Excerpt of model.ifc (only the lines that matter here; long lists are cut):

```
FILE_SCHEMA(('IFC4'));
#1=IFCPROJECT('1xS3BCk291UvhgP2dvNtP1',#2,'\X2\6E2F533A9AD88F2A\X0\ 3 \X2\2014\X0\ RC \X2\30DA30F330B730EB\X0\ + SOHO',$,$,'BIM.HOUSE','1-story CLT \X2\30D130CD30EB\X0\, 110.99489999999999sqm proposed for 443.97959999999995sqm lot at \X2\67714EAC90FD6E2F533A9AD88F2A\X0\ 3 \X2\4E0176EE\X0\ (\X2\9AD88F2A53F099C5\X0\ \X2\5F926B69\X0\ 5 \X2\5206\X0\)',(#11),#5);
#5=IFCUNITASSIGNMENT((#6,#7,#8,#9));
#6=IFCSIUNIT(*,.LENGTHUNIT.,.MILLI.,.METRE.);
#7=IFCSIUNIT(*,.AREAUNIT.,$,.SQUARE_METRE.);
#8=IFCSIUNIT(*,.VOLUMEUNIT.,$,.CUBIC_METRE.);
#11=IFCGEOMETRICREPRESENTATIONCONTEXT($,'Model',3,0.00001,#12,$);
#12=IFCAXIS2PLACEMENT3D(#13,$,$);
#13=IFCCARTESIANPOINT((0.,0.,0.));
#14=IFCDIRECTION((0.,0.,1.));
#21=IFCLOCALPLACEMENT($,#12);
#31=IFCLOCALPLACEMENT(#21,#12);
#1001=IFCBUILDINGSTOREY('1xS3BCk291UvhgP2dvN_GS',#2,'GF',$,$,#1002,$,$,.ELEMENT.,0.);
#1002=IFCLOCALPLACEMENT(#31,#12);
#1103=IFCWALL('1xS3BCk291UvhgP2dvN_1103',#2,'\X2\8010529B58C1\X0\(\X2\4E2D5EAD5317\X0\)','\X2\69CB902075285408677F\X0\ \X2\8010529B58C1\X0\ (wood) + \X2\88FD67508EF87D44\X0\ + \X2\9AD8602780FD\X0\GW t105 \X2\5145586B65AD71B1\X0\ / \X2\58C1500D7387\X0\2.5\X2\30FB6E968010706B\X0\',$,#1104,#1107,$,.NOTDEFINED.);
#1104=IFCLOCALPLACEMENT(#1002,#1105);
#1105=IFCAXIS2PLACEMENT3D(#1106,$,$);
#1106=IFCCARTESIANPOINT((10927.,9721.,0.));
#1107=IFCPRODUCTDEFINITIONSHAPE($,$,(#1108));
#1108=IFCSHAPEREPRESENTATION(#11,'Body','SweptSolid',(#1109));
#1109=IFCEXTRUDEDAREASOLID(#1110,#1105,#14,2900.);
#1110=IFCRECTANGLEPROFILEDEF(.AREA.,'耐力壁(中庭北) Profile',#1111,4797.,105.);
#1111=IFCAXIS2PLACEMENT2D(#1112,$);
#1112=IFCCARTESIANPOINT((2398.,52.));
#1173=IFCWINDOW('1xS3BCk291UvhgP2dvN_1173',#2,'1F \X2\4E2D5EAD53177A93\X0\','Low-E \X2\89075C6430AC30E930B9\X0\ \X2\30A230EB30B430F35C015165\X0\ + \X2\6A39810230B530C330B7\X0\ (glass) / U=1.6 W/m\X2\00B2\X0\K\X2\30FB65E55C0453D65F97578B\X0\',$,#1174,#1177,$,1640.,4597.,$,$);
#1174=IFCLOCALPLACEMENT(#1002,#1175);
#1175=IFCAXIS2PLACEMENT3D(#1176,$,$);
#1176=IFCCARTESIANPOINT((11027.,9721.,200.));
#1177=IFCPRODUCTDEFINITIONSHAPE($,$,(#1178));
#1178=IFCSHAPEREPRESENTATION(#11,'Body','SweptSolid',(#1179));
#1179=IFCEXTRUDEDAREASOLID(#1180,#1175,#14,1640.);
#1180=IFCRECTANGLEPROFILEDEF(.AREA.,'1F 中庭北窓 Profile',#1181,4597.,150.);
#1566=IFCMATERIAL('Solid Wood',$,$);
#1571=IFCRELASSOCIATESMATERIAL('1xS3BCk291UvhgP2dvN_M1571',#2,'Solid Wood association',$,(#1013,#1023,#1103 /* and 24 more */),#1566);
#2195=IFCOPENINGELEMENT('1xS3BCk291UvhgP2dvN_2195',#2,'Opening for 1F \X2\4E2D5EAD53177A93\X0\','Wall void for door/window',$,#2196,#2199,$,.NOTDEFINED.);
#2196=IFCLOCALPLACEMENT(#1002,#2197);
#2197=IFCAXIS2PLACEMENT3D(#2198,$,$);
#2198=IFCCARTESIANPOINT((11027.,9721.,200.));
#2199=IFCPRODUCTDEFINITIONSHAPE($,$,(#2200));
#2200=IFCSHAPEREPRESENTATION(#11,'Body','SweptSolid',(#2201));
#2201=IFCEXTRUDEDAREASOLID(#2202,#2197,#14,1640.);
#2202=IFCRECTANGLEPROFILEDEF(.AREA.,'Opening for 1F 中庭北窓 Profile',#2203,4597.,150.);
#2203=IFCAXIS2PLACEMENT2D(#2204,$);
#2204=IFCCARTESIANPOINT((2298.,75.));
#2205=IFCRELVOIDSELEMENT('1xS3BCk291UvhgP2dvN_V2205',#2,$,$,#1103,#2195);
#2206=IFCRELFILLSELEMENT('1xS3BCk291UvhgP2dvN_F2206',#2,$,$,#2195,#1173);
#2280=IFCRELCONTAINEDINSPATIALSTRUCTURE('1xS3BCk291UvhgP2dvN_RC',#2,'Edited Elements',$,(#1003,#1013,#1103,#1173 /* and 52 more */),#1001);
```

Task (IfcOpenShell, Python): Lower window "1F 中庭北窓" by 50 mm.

```python
import numpy as np
import ifcopenshell
import ifcopenshell.api.geometry
import ifcopenshell.util.placement
import ifcopenshell.util.unit

model = ifcopenshell.open("model.ifc")
unit_scale = ifcopenshell.util.unit.calculate_unit_scale(model)

window = model.by_guid("1xS3BCk291UvhgP2dvN_1173")
opening = window.FillsVoids[0].RelatingOpeningElement
dz = -50.0

shift = np.array([0.0, 0.0, dz])
# The window is not placed relative to its opening, so move both.
for product in (opening, window):
    matrix = ifcopenshell.util.placement.get_local_placement(product.ObjectPlacement)
    matrix[:3, 3] += shift
    ifcopenshell.api.geometry.edit_object_placement(model, product=product, matrix=matrix, is_si=False)

print(f"moved by {dz * unit_scale:+.3f} m")

model.write("model_edited.ifc")
```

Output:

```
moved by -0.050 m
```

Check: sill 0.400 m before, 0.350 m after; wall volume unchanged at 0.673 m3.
